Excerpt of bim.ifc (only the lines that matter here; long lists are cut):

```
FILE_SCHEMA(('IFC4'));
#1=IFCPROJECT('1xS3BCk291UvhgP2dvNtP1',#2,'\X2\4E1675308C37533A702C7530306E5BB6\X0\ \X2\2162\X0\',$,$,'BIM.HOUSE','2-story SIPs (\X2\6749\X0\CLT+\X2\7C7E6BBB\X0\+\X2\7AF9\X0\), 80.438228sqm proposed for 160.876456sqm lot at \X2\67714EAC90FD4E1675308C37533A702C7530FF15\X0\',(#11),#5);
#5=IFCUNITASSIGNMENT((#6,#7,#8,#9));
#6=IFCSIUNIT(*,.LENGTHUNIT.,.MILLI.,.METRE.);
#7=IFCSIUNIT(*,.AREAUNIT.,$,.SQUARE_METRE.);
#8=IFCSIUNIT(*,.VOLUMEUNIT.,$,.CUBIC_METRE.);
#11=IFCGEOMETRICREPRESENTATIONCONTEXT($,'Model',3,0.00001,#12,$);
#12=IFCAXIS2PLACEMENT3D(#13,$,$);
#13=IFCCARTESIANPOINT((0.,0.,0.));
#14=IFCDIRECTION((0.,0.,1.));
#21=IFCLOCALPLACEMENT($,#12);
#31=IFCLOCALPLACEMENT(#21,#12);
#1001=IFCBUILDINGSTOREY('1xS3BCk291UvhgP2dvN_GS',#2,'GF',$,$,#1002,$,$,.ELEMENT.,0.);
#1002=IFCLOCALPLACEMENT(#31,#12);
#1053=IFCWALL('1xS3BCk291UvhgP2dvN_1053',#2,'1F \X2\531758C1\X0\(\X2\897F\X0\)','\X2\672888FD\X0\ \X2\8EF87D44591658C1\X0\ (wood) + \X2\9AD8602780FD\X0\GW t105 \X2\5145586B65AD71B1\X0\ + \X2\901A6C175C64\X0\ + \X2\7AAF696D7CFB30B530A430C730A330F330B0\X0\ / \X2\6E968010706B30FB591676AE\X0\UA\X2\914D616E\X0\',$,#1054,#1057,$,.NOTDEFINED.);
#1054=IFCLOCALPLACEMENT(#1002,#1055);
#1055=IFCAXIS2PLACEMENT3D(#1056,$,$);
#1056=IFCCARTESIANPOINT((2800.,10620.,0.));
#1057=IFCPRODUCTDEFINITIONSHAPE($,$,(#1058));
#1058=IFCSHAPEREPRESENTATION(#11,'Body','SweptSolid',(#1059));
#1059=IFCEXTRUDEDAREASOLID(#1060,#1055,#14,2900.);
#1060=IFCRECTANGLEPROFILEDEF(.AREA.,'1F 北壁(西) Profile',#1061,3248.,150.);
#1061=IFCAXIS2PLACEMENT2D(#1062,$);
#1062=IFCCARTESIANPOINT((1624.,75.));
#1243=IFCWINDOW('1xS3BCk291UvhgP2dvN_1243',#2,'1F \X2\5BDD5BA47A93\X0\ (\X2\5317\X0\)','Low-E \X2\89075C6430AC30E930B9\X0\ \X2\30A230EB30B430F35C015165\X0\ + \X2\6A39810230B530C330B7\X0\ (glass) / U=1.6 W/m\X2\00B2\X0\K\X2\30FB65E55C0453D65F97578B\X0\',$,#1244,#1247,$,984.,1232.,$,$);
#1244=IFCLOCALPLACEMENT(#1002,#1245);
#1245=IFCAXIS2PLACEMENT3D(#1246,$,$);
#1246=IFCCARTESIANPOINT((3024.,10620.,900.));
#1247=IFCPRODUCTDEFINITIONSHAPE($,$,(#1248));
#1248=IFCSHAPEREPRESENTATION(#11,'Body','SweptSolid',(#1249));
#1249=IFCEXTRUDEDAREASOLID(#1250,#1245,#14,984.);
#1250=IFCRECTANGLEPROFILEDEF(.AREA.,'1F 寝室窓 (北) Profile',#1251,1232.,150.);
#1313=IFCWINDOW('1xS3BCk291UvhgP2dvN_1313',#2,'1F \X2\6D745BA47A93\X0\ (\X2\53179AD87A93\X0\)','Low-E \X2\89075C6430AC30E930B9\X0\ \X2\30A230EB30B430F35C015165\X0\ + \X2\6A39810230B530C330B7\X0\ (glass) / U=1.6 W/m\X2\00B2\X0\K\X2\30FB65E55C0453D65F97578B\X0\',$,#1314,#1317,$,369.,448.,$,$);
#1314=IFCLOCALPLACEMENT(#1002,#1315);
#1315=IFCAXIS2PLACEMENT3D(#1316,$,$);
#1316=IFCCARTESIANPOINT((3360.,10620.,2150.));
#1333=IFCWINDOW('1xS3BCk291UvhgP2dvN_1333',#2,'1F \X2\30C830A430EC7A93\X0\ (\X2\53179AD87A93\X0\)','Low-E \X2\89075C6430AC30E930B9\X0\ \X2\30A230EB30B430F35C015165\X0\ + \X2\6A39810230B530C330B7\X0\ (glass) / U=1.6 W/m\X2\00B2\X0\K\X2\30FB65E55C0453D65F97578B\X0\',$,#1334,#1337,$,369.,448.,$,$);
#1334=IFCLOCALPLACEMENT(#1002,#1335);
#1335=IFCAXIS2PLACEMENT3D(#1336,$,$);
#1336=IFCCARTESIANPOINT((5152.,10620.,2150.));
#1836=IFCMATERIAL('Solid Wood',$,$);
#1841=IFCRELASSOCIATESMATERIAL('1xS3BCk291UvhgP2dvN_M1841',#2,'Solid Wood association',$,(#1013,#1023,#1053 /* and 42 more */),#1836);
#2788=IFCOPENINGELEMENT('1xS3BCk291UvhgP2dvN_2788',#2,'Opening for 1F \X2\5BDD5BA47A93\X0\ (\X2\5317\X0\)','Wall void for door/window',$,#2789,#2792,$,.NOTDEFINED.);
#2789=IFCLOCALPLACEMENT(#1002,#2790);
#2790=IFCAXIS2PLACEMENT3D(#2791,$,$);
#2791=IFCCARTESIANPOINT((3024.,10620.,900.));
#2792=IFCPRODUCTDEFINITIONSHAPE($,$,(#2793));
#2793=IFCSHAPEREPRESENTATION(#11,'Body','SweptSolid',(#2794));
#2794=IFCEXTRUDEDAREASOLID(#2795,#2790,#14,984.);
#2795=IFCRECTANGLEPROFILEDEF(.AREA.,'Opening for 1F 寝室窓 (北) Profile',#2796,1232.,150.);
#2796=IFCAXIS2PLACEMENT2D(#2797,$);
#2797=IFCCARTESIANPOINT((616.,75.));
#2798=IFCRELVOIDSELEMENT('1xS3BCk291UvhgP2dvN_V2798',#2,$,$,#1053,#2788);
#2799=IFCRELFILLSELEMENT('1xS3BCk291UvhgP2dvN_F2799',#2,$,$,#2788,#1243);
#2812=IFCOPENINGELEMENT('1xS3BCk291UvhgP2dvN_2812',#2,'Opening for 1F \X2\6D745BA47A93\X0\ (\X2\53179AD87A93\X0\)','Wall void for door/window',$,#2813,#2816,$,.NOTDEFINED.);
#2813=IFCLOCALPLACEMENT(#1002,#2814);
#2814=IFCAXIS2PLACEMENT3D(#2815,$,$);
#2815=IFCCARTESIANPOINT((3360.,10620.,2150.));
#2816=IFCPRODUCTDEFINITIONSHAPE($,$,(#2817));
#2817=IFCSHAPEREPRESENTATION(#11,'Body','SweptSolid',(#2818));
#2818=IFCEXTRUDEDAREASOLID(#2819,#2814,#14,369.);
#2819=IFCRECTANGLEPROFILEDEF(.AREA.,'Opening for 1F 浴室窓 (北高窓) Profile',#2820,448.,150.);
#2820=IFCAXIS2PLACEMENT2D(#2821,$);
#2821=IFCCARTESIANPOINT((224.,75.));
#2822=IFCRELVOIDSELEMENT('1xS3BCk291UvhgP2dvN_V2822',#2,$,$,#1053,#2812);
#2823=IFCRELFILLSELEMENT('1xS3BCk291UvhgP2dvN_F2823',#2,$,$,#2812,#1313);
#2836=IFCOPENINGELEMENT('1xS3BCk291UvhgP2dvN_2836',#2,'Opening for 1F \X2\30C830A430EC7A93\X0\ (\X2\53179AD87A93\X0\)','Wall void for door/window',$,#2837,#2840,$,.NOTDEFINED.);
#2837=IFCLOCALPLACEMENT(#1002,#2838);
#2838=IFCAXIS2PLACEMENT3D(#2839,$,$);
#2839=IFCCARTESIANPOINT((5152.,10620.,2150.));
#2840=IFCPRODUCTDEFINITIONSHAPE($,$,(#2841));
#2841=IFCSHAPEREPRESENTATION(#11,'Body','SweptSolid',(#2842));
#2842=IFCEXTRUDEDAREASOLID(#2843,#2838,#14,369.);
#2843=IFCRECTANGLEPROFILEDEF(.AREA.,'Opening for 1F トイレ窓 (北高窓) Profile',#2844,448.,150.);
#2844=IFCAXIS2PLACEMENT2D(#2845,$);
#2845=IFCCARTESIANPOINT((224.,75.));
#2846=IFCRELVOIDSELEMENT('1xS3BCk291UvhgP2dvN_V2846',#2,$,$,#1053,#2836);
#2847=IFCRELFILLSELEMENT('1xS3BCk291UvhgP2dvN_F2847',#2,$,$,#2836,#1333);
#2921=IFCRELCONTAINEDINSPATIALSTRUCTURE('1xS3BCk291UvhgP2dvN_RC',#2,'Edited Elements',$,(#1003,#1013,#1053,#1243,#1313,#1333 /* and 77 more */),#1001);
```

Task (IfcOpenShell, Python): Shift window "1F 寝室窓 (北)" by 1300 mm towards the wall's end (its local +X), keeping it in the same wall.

```python
import ifcopenshell
import ifcopenshell.api.geometry
import ifcopenshell.util.placement

model = ifcopenshell.open("bim.ifc")

window = model.by_id(1243)
opening = window.FillsVoids[0].RelatingOpeningElement
wall = opening.VoidsElements[0].RelatingBuildingElement

wall_matrix = ifcopenshell.util.placement.get_local_placement(wall.ObjectPlacement)
shift = wall_matrix[:3, 0] * 1300.0
before = ifcopenshell.util.placement.get_local_placement(window.ObjectPlacement)[:3, 3].copy()

# The window is not placed relative to its opening, so move both.
for product in (opening, window):
    matrix = ifcopenshell.util.placement.get_local_placement(product.ObjectPlacement)
    matrix[:3, 3] += shift
    ifcopenshell.api.geometry.edit_object_placement(model, product=product, matrix=matrix, is_si=False)

after = ifcopenshell.util.placement.get_local_placement(window.ObjectPlacement)[:3, 3]
print("window moved by", (after - before).round(3) + 0.0)

model.write("bim-out.ifc")
```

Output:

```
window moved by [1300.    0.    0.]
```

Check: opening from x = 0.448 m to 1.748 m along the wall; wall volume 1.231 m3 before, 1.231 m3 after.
